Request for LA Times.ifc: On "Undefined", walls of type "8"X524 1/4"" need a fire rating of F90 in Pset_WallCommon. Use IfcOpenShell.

First a look at what the model holds.

```python
import ifcopenshell
import ifcopenshell.util.element

model = ifcopenshell.open("LA Times.ifc")
print(model.schema)
storey = next(s for s in model.by_type("IfcBuildingStorey") if s.Name == "Undefined")
walls = [e for e in ifcopenshell.util.element.get_decomposition(storey) if e.is_a("IfcWall")]
seen = {}
for e in walls:
    element_type = ifcopenshell.util.element.get_type(e)
    key = (element_type.Name if element_type != e and element_type else None, ifcopenshell.util.element.get_pset(e, "Pset_WallCommon", "FireRating"))
    seen[key] = seen.get(key, 0) + 1
for (name, value), count in sorted(seen.items(), key=str):
    print(count, "x", name, "|", value)
```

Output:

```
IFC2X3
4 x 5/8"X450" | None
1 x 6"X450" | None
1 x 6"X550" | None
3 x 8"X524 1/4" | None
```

```python
import ifcopenshell
import ifcopenshell.api.pset
import ifcopenshell.util.element

model = ifcopenshell.open("LA Times.ifc")

storey = next(s for s in model.by_type("IfcBuildingStorey") if s.Name == "Undefined")
walls = [e for e in ifcopenshell.util.element.get_decomposition(storey) if e.is_a("IfcWall")]

count = 0
for e in walls:
    element_type = ifcopenshell.util.element.get_type(e)
    if element_type in (None, e) or element_type.Name != '8"X524 1/4"':
        continue
    found = ifcopenshell.util.element.get_pset(e, "Pset_WallCommon", should_inherit=False)
    if found:
        pset = model.by_id(found["id"])
        if len(ifcopenshell.util.element.get_elements_by_pset(pset)) > 1:
            pset = ifcopenshell.api.pset.unshare_pset(model, products=[e], pset=pset)[0]
    else:
        pset = ifcopenshell.api.pset.add_pset(model, product=e, name="Pset_WallCommon")
    ifcopenshell.api.pset.edit_pset(model, pset=pset, properties={"FireRating": "F90"})
    count += 1

print(count, "walls updated")

model.write("LA Times_updated.ifc")
```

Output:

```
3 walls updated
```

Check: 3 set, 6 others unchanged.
